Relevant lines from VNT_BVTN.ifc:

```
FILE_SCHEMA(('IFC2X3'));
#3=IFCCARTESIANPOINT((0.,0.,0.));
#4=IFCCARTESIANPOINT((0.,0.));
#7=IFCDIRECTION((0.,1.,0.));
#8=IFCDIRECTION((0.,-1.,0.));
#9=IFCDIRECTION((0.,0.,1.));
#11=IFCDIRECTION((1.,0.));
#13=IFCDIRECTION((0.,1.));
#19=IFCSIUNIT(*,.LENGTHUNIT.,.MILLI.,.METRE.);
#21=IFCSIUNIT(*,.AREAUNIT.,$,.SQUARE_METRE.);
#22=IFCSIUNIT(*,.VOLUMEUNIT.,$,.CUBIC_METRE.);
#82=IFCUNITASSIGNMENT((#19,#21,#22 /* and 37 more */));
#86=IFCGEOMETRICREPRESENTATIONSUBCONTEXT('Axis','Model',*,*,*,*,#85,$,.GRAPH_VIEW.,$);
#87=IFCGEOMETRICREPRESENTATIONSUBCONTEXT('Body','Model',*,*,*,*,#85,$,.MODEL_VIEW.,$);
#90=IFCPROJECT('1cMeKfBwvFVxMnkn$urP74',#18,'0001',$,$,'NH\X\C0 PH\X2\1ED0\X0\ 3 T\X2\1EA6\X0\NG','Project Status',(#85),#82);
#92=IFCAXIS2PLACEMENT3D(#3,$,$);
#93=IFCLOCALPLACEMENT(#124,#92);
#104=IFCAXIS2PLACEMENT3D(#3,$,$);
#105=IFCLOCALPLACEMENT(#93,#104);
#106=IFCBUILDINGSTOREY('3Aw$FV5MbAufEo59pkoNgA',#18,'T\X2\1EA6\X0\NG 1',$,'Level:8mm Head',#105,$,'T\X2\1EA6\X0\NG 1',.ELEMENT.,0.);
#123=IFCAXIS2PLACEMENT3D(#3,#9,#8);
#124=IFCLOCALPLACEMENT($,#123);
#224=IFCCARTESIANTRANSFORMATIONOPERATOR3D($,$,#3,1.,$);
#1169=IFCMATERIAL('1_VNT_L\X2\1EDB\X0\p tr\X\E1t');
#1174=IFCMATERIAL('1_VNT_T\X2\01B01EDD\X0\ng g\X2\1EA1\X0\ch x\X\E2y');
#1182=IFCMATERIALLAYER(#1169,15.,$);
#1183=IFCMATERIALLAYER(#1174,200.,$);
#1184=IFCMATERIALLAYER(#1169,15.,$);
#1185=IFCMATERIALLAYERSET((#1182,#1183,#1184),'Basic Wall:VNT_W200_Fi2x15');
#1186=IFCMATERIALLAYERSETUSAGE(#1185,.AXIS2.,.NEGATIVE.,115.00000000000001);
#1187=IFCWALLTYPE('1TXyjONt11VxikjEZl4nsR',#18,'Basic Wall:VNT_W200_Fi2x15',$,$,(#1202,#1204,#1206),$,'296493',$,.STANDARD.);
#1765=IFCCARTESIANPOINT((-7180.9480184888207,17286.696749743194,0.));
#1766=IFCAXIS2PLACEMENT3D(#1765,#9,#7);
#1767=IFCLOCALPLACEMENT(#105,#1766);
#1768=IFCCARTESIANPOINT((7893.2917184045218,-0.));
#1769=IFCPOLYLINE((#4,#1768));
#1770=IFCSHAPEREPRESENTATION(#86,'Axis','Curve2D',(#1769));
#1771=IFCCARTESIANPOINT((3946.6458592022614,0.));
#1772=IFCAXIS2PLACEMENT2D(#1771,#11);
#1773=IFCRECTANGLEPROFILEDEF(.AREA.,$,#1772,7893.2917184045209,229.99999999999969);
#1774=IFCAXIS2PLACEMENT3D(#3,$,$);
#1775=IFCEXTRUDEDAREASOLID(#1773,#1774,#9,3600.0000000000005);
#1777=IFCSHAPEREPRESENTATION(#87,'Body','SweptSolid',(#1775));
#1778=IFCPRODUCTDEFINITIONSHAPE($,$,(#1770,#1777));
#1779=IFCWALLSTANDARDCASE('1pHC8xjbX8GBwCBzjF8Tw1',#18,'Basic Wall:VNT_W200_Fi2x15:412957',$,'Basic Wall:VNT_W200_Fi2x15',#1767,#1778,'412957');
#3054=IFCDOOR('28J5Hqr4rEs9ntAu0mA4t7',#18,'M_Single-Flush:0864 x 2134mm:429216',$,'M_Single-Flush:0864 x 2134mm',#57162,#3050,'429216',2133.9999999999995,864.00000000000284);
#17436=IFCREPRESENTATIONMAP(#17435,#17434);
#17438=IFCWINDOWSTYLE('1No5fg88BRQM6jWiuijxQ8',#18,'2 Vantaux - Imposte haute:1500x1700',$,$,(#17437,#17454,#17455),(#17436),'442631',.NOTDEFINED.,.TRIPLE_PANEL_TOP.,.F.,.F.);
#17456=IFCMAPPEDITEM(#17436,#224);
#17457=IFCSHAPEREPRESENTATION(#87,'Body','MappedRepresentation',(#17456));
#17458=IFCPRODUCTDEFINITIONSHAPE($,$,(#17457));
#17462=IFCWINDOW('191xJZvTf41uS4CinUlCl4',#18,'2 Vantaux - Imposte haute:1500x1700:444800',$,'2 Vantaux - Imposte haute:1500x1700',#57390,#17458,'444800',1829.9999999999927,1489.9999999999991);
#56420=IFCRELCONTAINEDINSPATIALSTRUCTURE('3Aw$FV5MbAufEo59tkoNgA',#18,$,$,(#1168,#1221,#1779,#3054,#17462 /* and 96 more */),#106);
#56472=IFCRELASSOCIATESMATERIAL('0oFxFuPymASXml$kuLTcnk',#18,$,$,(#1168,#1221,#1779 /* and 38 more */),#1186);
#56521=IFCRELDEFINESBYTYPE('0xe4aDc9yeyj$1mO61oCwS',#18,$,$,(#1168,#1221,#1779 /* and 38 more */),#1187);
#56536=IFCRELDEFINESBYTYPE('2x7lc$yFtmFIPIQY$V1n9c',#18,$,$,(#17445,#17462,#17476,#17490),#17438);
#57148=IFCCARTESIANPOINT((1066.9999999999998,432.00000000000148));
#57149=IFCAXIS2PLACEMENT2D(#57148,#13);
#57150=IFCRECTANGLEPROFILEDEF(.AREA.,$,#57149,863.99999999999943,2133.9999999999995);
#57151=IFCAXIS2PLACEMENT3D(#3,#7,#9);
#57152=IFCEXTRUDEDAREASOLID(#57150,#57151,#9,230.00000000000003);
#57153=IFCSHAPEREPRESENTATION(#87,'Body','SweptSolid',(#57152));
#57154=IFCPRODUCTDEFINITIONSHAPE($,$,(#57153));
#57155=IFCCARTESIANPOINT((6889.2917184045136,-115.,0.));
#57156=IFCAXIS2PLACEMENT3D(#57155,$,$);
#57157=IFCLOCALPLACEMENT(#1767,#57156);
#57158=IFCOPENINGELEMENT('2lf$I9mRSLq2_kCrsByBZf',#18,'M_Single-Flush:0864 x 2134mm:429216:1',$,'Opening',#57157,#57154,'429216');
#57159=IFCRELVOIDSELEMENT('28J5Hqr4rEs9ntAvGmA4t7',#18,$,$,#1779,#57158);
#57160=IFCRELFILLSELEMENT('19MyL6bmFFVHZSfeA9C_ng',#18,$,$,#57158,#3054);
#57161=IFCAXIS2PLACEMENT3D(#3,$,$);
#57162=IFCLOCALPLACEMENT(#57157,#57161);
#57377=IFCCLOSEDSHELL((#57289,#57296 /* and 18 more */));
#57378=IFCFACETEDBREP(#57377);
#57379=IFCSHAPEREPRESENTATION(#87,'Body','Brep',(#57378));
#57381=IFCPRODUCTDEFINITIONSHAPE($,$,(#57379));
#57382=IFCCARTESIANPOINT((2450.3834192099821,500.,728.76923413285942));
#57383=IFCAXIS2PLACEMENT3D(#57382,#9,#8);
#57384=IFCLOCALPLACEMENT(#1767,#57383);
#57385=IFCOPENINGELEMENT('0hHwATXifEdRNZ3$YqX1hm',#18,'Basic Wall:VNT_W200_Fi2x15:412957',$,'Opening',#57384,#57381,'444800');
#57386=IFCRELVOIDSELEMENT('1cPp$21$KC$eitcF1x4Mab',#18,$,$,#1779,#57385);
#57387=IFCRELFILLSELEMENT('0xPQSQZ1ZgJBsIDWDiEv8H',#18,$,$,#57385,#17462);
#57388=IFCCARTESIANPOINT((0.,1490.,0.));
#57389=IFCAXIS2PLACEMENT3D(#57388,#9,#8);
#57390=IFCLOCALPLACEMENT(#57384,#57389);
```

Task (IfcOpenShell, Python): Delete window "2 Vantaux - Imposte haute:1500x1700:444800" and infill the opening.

```python
import ifcopenshell
import ifcopenshell.api.feature
import ifcopenshell.api.root
import ifcopenshell.geom
import ifcopenshell.util.shape

model = ifcopenshell.open("VNT_BVTN.ifc")
settings = ifcopenshell.geom.settings()


def volume(element):
    """Net volume in cubic metres, openings subtracted."""
    shape = ifcopenshell.geom.create_shape(settings, element)
    return ifcopenshell.util.shape.get_volume(shape.geometry)


window = model.by_id(17462)
opening = window.FillsVoids[0].RelatingOpeningElement
wall = opening.VoidsElements[0].RelatingBuildingElement
before = volume(wall)

ifcopenshell.api.root.remove_product(model, product=window)
ifcopenshell.api.feature.remove_feature(model, feature=opening)

after = volume(wall)

print(f"wall volume {before:.3f} -> {after:.3f} m3")

model.write("VNT_BVTN_updated.ifc")
```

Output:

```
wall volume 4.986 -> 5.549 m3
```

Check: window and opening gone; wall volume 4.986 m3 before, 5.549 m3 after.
